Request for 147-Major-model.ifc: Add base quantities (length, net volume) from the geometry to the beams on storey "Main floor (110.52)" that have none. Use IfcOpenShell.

First a look at what the model holds.

```python
import ifcopenshell
import ifcopenshell.util.element
import ifcopenshell.util.unit

model = ifcopenshell.open("147-Major-model.ifc")
print(model.schema)
for unit_type in ("LENGTHUNIT", "AREAUNIT", "VOLUMEUNIT"):
    print(unit_type, ifcopenshell.util.unit.calculate_unit_scale(model, unit_type))
storey = next(s for s in model.by_type("IfcBuildingStorey") if s.Name == "Main floor (110.52)")
beams = [e for e in ifcopenshell.util.element.get_decomposition(storey) if e.is_a("IfcBeam")]
for e in sorted(beams, key=lambda e: e.id()):
    print(e.id(), e.is_a(), e.Name, list(ifcopenshell.util.element.get_psets(e, qtos_only=True)), sep=" | ")
```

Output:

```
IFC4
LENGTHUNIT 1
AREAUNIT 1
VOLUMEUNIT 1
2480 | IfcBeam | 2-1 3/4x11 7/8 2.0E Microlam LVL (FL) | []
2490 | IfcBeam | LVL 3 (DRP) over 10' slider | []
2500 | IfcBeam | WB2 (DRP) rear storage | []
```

```python
import ifcopenshell
import ifcopenshell.api.pset
import ifcopenshell.geom
import ifcopenshell.util.element
import ifcopenshell.util.shape
import ifcopenshell.util.unit

model = ifcopenshell.open("147-Major-model.ifc")
unit_scale = ifcopenshell.util.unit.calculate_unit_scale(model)
volume_scale = ifcopenshell.util.unit.calculate_unit_scale(model, "VOLUMEUNIT")
settings = ifcopenshell.geom.settings()

storey = next(s for s in model.by_type("IfcBuildingStorey") if s.Name == "Main floor (110.52)")
beams = [e for e in ifcopenshell.util.element.get_decomposition(storey) if e.is_a("IfcBeam")]

for e in sorted(beams, key=lambda e: e.id()):
    if ifcopenshell.util.element.get_psets(e, qtos_only=True, should_inherit=False):
        continue
    # Geometry comes back in metres, in the element's own axes.
    shape = ifcopenshell.geom.create_shape(settings, e)
    values = {
        "Length": ifcopenshell.util.shape.get_max_xyz(shape.geometry) / unit_scale,
        "NetVolume": ifcopenshell.util.shape.get_volume(shape.geometry) / volume_scale,
    }
    qto = ifcopenshell.api.pset.add_qto(model, product=e, name="Qto_BeamBaseQuantities")
    ifcopenshell.api.pset.edit_qto(model, qto=qto, properties=values)
    print(e.id(), {k: round(v, 3) for k, v in values.items()})

model.write("147-Major-model_v2.ifc")
```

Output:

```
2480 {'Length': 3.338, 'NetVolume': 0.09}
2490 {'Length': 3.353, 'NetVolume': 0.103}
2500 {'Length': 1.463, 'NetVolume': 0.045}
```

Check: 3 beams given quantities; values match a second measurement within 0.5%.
